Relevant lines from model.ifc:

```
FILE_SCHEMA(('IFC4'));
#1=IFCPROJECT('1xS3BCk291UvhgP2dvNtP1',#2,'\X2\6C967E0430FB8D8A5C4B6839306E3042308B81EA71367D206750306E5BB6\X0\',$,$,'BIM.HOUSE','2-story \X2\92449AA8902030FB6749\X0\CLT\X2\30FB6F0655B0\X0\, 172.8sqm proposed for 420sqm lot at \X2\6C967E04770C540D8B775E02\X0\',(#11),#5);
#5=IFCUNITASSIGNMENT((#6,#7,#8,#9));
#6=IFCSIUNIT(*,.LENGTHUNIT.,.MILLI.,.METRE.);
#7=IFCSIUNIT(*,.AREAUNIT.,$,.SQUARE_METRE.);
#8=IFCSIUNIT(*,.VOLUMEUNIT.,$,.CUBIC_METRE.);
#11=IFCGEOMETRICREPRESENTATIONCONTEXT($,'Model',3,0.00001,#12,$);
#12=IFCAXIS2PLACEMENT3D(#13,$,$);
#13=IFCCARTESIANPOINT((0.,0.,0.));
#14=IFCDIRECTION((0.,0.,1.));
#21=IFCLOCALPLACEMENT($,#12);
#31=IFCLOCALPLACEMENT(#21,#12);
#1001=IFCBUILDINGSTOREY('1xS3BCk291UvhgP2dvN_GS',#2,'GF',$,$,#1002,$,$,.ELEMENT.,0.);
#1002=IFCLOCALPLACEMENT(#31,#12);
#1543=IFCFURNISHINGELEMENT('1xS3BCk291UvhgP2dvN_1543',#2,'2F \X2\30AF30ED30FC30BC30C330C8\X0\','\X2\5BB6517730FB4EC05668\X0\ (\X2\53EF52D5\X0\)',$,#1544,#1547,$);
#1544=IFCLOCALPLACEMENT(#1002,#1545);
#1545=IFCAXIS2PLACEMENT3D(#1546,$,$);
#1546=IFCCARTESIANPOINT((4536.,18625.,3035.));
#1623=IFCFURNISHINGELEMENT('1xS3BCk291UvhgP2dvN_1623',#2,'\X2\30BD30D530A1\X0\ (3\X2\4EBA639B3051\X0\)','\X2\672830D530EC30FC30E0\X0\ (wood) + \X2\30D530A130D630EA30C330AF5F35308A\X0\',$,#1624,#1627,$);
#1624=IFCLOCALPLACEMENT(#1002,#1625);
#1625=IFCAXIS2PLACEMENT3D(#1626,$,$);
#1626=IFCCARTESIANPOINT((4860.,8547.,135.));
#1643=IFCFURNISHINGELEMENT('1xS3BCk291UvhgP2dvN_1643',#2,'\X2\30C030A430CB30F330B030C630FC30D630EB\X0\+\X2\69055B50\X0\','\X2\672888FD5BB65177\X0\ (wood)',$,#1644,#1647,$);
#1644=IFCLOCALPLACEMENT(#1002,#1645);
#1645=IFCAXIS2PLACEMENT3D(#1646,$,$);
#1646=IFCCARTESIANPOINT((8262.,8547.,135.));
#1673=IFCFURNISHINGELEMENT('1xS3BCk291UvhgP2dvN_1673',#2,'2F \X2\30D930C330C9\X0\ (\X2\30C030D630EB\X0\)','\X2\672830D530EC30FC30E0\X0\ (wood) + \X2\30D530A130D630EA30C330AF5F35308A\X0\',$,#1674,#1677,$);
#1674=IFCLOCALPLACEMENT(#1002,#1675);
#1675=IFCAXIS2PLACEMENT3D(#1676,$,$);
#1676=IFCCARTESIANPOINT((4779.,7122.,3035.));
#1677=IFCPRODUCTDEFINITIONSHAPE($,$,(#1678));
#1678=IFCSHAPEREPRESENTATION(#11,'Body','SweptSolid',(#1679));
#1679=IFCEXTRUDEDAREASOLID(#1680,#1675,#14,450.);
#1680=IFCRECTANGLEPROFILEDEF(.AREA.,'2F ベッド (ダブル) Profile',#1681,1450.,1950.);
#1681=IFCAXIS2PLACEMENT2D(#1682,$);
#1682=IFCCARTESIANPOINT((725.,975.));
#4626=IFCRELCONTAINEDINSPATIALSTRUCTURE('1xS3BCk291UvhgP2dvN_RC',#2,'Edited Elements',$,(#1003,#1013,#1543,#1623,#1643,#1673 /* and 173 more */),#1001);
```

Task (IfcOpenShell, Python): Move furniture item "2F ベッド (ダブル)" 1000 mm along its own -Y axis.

```python
import ifcopenshell
import ifcopenshell.api.geometry
import ifcopenshell.util.placement

model = ifcopenshell.open("model.ifc")

item = model.by_guid("1xS3BCk291UvhgP2dvN_1673")
matrix = ifcopenshell.util.placement.get_local_placement(item.ObjectPlacement)
matrix[:3, 3] -= matrix[:3, 1] * 1000.0
ifcopenshell.api.geometry.edit_object_placement(model, product=item, matrix=matrix, is_si=False)

print(ifcopenshell.util.placement.get_local_placement(item.ObjectPlacement).round(3) + 0.0)

model.write("model_updated.ifc")
```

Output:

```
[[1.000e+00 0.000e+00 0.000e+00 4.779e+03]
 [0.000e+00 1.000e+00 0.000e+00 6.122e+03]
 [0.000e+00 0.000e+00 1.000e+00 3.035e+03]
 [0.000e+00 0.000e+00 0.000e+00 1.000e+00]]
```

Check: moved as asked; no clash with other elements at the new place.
